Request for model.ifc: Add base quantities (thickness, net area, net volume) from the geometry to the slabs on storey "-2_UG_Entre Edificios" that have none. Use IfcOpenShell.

First a look at what the model holds.

```python
import ifcopenshell
import ifcopenshell.util.element
import ifcopenshell.util.unit

model = ifcopenshell.open("model.ifc")
print(model.schema)
for unit_type in ("LENGTHUNIT", "AREAUNIT", "VOLUMEUNIT"):
    print(unit_type, ifcopenshell.util.unit.calculate_unit_scale(model, unit_type))
storey = next(s for s in model.by_type("IfcBuildingStorey") if s.Name == "-2_UG_Entre Edificios")
slabs = [e for e in ifcopenshell.util.element.get_decomposition(storey) if e.is_a("IfcSlab")]
for e in sorted(slabs, key=lambda e: e.id()):
    print(e.id(), e.is_a(), e.Name, list(ifcopenshell.util.element.get_psets(e, qtos_only=True)), sep=" | ")
```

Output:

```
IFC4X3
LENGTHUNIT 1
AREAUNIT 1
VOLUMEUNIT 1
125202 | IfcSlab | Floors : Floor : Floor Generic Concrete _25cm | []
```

```python
import ifcopenshell
import ifcopenshell.api.pset
import ifcopenshell.geom
import ifcopenshell.util.element
import ifcopenshell.util.shape
import ifcopenshell.util.unit

model = ifcopenshell.open("model.ifc")
unit_scale = ifcopenshell.util.unit.calculate_unit_scale(model)
area_scale = ifcopenshell.util.unit.calculate_unit_scale(model, "AREAUNIT")
volume_scale = ifcopenshell.util.unit.calculate_unit_scale(model, "VOLUMEUNIT")
settings = ifcopenshell.geom.settings()

storey = next(s for s in model.by_type("IfcBuildingStorey") if s.Name == "-2_UG_Entre Edificios")
slabs = [e for e in ifcopenshell.util.element.get_decomposition(storey) if e.is_a("IfcSlab")]

for e in sorted(slabs, key=lambda e: e.id()):
    if ifcopenshell.util.element.get_psets(e, qtos_only=True, should_inherit=False):
        continue
    # Geometry comes back in metres, in the element's own axes.
    shape = ifcopenshell.geom.create_shape(settings, e)
    values = {
        "Width": ifcopenshell.util.shape.get_z(shape.geometry) / unit_scale,
        "NetArea": ifcopenshell.util.shape.get_footprint_area(shape.geometry) / area_scale,
        "NetVolume": ifcopenshell.util.shape.get_volume(shape.geometry) / volume_scale,
    }
    qto = ifcopenshell.api.pset.add_qto(model, product=e, name="Qto_SlabBaseQuantities")
    ifcopenshell.api.pset.edit_qto(model, qto=qto, properties=values)
    print(e.id(), {k: round(v, 3) for k, v in values.items()})

model.write("model_rev.ifc")
```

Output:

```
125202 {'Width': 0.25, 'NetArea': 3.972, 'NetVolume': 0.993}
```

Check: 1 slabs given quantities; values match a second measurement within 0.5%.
